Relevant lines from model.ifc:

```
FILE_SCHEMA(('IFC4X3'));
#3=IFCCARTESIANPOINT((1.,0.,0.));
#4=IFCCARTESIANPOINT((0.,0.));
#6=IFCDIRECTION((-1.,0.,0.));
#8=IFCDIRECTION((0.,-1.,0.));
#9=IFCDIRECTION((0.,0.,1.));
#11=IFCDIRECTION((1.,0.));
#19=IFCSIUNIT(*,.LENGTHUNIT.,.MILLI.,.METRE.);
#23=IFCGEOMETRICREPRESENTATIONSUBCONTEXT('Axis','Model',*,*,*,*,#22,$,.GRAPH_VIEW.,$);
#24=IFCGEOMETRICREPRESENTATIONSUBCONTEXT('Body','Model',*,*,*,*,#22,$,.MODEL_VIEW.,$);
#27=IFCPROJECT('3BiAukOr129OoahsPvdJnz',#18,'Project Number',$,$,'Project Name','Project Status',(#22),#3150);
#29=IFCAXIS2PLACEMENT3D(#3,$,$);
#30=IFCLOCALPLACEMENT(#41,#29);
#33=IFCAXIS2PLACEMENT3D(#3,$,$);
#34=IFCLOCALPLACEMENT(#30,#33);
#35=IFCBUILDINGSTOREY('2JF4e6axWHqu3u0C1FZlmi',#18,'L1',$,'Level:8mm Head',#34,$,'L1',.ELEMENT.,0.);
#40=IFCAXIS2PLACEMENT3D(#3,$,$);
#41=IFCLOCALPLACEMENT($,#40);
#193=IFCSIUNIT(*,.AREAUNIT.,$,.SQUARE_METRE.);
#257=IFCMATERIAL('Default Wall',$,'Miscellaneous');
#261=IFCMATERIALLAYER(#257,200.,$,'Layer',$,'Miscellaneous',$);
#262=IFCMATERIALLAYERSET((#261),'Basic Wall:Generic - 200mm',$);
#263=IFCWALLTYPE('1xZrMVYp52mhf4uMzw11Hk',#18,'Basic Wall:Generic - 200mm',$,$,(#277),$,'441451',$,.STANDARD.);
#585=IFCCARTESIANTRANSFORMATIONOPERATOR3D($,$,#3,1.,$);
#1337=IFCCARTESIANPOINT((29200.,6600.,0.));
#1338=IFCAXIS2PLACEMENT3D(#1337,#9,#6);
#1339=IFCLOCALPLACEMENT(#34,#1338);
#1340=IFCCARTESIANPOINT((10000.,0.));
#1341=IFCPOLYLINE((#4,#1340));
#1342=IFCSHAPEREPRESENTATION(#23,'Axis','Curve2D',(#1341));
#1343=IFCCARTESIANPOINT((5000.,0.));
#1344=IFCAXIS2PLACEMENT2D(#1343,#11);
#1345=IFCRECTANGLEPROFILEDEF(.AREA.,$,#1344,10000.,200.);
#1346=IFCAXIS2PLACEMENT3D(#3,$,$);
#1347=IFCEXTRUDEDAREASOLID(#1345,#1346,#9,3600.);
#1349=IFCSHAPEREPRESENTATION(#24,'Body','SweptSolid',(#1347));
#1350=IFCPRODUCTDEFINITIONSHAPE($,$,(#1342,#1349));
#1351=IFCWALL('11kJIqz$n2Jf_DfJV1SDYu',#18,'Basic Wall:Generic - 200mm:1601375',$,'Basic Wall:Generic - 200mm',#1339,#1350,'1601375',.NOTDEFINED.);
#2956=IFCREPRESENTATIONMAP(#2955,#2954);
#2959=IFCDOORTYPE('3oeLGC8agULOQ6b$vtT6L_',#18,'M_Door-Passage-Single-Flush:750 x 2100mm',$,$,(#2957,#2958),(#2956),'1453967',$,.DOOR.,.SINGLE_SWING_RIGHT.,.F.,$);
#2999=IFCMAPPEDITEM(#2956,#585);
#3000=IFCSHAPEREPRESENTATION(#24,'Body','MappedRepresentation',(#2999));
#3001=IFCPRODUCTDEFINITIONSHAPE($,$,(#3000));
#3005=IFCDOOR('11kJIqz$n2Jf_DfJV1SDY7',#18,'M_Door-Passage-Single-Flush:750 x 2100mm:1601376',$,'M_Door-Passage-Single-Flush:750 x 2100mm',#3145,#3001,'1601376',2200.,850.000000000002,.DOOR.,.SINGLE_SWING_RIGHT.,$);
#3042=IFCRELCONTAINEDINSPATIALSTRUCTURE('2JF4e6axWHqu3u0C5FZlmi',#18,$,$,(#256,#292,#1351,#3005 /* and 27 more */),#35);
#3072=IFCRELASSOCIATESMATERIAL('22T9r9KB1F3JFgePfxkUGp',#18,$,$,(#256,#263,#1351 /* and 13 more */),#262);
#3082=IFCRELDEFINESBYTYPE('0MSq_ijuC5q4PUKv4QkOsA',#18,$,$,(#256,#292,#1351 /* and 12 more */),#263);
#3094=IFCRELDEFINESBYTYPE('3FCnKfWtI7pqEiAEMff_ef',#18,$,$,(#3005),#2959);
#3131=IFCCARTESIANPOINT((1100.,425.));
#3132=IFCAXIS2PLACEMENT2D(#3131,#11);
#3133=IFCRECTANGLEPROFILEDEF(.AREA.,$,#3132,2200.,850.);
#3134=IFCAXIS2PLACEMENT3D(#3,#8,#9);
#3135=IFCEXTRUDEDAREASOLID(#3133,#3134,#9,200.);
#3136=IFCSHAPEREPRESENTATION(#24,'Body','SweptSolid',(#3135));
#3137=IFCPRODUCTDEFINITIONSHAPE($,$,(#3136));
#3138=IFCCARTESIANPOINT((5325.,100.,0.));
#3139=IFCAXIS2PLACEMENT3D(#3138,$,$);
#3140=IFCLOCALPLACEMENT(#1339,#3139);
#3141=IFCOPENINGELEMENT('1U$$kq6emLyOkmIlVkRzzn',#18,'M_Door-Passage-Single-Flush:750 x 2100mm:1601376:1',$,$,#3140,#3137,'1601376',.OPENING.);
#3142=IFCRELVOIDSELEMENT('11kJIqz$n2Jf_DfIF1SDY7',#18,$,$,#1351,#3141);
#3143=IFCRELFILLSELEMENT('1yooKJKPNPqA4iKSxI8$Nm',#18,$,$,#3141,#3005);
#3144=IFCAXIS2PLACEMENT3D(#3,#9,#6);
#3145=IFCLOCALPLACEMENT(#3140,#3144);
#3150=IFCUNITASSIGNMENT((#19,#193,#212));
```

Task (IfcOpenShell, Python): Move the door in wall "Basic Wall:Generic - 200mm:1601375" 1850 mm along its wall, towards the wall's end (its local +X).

```python
import ifcopenshell
import ifcopenshell.api.geometry
import ifcopenshell.util.placement
import ifcopenshell.util.unit

model = ifcopenshell.open("model.ifc")
unit_scale = ifcopenshell.util.unit.calculate_unit_scale(model)

door = model.by_guid("11kJIqz$n2Jf_DfJV1SDY7")
opening = door.FillsVoids[0].RelatingOpeningElement
wall = opening.VoidsElements[0].RelatingBuildingElement

wall_matrix = ifcopenshell.util.placement.get_local_placement(wall.ObjectPlacement)
shift = wall_matrix[:3, 0] * 1.85 / unit_scale
before = ifcopenshell.util.placement.get_local_placement(door.ObjectPlacement)[:3, 3].copy()

# The door is placed relative to its opening, so it follows when the opening moves.
matrix = ifcopenshell.util.placement.get_local_placement(opening.ObjectPlacement)
matrix[:3, 3] += shift
ifcopenshell.api.geometry.edit_object_placement(
    model, product=opening, matrix=matrix, is_si=False, should_transform_children=True
)

after = ifcopenshell.util.placement.get_local_placement(door.ObjectPlacement)[:3, 3]
print("door moved by", (after - before).round(3) + 0.0)

model.write("model_v2.ifc")
```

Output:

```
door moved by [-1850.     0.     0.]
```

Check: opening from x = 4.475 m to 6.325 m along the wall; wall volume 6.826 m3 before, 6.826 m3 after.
